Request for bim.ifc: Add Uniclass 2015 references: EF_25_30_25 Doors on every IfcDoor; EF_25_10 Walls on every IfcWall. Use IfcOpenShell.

First a look at what the model holds.

```python
import ifcopenshell

model = ifcopenshell.open("bim.ifc")
print(model.schema)
print("classifications:", [c.Name for c in model.by_type("IfcClassification")])
for ifc_class in ("IfcDoor", "IfcRoof", "IfcStair", "IfcWall", "IfcWindow"):
    print(ifc_class, len(model.by_type(ifc_class)))
```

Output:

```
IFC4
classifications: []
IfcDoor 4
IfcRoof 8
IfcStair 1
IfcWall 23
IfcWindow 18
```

```python
import ifcopenshell
import ifcopenshell.api.classification

model = ifcopenshell.open("bim.ifc")

system = ifcopenshell.api.classification.add_classification(model, classification="Uniclass 2015")

codes = {
    "IfcDoor": ("EF_25_30_25", "Doors"),
    "IfcWall": ("EF_25_10", "Walls"),
}
for ifc_class, (code, name) in codes.items():
    products = model.by_type(ifc_class)
    ifcopenshell.api.classification.add_reference(
        model, products=products, classification=system, identification=code, name=name
    )
    print(code, len(products))

model.write("bim-out.ifc")
```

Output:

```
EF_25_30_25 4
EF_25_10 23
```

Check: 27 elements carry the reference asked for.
